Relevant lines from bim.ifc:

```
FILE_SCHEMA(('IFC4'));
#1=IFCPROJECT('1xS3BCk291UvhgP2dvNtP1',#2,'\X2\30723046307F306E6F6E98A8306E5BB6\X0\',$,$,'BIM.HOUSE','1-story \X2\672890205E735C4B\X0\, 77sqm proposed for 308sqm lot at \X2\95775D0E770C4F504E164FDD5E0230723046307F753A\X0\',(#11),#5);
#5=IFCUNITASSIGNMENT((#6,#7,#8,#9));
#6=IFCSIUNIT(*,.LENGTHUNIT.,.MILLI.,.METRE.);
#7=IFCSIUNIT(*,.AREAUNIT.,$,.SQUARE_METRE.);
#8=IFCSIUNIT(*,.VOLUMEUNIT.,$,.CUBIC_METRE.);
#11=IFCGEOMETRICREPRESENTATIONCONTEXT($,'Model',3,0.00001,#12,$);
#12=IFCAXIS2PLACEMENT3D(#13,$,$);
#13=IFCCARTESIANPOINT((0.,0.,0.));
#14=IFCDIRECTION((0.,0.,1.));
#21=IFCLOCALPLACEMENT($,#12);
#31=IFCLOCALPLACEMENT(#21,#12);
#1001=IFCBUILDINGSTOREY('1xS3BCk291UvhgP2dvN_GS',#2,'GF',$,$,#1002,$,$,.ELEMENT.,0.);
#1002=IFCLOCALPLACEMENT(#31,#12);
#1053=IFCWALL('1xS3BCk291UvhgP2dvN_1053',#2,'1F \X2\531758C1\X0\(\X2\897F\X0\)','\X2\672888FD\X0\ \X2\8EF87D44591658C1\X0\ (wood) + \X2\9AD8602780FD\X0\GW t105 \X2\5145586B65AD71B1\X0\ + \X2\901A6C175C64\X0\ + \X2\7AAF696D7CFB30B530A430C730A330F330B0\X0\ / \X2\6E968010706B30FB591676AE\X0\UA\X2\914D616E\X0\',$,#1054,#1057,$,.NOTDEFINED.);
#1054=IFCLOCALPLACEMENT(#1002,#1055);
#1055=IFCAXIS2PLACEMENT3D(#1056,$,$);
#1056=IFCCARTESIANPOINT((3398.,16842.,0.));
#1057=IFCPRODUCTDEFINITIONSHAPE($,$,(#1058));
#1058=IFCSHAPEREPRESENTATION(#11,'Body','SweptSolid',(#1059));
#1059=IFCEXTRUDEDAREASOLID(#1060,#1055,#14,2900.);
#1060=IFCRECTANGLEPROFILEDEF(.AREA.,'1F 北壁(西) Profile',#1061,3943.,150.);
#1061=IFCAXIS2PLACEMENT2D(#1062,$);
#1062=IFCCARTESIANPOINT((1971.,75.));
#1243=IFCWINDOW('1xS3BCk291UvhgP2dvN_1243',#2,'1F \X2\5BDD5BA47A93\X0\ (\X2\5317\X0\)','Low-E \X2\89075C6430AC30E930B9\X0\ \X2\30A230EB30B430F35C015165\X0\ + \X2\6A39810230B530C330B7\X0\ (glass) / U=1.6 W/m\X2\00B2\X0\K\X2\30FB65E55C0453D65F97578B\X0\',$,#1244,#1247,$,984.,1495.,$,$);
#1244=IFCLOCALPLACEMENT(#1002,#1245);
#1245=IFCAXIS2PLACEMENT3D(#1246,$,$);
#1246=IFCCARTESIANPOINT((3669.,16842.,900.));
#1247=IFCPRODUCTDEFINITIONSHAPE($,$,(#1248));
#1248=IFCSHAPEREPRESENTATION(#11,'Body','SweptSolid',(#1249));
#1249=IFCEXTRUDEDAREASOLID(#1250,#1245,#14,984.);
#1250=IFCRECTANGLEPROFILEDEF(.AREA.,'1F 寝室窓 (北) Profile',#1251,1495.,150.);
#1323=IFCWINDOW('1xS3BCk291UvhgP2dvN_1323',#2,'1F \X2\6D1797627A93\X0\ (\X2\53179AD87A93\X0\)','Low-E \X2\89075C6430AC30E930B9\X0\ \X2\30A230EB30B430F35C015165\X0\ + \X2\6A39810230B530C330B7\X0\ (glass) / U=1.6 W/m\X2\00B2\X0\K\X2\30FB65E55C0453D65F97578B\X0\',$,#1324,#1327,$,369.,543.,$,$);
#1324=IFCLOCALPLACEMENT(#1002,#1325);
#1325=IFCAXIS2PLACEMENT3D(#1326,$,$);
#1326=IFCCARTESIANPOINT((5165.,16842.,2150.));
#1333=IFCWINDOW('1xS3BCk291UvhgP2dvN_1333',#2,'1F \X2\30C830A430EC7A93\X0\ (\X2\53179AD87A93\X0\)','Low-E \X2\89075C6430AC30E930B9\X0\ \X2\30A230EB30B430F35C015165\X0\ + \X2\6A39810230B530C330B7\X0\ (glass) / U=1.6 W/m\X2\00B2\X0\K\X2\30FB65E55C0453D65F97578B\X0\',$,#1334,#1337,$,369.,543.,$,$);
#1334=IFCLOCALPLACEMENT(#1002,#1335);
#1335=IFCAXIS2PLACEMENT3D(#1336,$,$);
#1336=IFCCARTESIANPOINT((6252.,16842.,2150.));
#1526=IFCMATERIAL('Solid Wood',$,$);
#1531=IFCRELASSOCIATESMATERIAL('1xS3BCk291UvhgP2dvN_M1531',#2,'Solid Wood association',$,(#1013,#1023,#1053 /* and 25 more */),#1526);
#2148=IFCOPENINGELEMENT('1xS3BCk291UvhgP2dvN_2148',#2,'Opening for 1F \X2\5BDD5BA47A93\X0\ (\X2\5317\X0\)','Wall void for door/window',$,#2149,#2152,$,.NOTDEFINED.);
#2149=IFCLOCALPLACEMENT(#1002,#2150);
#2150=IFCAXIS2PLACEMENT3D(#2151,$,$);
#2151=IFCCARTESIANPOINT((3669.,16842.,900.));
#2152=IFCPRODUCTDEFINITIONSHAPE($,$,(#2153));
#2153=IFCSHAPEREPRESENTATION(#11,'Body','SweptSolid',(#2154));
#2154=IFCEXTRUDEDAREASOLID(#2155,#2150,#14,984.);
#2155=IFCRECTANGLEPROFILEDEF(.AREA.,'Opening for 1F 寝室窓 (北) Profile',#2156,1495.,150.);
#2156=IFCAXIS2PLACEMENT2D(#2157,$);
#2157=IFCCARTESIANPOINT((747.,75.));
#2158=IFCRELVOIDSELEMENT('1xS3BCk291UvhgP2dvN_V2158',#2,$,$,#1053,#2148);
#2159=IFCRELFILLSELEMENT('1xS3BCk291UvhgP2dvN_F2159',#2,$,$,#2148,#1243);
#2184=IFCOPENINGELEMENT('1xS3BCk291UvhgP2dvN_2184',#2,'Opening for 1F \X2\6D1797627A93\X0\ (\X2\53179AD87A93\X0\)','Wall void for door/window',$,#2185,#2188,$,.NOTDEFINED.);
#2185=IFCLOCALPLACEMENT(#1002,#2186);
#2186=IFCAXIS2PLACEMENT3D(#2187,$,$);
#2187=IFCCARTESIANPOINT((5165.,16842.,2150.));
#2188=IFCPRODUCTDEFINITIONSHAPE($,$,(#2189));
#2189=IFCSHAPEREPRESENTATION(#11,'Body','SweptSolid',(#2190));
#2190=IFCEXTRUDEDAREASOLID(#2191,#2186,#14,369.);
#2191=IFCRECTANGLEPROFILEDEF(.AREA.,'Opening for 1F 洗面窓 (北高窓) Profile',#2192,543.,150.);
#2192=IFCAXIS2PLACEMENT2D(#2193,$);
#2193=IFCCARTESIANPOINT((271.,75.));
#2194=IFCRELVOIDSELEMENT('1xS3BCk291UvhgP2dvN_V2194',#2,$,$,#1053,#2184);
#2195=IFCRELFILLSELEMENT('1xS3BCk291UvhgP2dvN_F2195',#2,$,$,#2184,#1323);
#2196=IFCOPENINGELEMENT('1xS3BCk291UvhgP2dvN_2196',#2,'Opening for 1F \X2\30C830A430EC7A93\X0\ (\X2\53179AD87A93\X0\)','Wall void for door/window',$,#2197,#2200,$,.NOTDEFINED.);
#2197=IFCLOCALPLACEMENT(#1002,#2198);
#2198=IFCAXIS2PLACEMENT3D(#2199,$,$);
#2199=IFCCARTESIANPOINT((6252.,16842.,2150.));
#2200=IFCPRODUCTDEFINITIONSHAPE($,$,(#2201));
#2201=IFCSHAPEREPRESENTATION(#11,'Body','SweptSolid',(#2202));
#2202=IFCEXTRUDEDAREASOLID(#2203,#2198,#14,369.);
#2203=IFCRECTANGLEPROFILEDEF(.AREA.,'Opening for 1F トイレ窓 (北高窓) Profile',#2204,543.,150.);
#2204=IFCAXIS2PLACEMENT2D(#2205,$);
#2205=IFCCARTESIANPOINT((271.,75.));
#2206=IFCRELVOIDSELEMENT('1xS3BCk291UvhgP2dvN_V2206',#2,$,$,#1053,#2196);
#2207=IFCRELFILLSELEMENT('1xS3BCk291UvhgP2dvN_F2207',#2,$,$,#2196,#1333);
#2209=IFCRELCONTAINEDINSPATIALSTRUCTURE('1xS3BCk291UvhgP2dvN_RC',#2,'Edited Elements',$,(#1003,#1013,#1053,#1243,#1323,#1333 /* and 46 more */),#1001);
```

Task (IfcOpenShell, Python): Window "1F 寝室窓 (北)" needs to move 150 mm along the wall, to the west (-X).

```python
import ifcopenshell
import ifcopenshell.api.geometry
import ifcopenshell.util.placement

model = ifcopenshell.open("bim.ifc")

window = model.by_id(1243)
opening = window.FillsVoids[0].RelatingOpeningElement
wall = opening.VoidsElements[0].RelatingBuildingElement

wall_matrix = ifcopenshell.util.placement.get_local_placement(wall.ObjectPlacement)
shift = wall_matrix[:3, 0] * -150.0
before = ifcopenshell.util.placement.get_local_placement(window.ObjectPlacement)[:3, 3].copy()

# The window is not placed relative to its opening, so move both.
for product in (opening, window):
    matrix = ifcopenshell.util.placement.get_local_placement(product.ObjectPlacement)
    matrix[:3, 3] += shift
    ifcopenshell.api.geometry.edit_object_placement(model, product=product, matrix=matrix, is_si=False)

after = ifcopenshell.util.placement.get_local_placement(window.ObjectPlacement)[:3, 3]
print("window moved by", (after - before).round(3) + 0.0)

model.write("bim_rev.ifc")
```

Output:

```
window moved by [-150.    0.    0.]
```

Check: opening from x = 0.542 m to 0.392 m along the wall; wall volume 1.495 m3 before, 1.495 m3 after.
